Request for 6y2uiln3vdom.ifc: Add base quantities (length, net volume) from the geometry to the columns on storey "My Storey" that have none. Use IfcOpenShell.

First a look at what the model holds.

```python
import ifcopenshell
import ifcopenshell.util.element
import ifcopenshell.util.unit

model = ifcopenshell.open("6y2uiln3vdom.ifc")
print(model.schema)
for unit_type in ("LENGTHUNIT", "AREAUNIT", "VOLUMEUNIT"):
    print(unit_type, ifcopenshell.util.unit.calculate_unit_scale(model, unit_type))
storey = next(s for s in model.by_type("IfcBuildingStorey") if s.Name == "My Storey")
columns = [e for e in ifcopenshell.util.element.get_decomposition(storey) if e.is_a("IfcColumn")]
for e in sorted(columns, key=lambda e: e.id()):
    print(e.id(), e.is_a(), e.Name, list(ifcopenshell.util.element.get_psets(e, qtos_only=True)), sep=" | ")
```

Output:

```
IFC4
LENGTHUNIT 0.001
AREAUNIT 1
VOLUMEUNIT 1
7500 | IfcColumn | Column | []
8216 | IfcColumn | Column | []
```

```python
import ifcopenshell
import ifcopenshell.api.pset
import ifcopenshell.geom
import ifcopenshell.util.element
import ifcopenshell.util.shape
import ifcopenshell.util.unit

model = ifcopenshell.open("6y2uiln3vdom.ifc")
unit_scale = ifcopenshell.util.unit.calculate_unit_scale(model)
volume_scale = ifcopenshell.util.unit.calculate_unit_scale(model, "VOLUMEUNIT")
settings = ifcopenshell.geom.settings()

storey = next(s for s in model.by_type("IfcBuildingStorey") if s.Name == "My Storey")
columns = [e for e in ifcopenshell.util.element.get_decomposition(storey) if e.is_a("IfcColumn")]

for e in sorted(columns, key=lambda e: e.id()):
    if ifcopenshell.util.element.get_psets(e, qtos_only=True, should_inherit=False):
        continue
    # Geometry comes back in metres, in the element's own axes.
    shape = ifcopenshell.geom.create_shape(settings, e)
    values = {
        "Length": ifcopenshell.util.shape.get_z(shape.geometry) / unit_scale,
        "NetVolume": ifcopenshell.util.shape.get_volume(shape.geometry) / volume_scale,
    }
    qto = ifcopenshell.api.pset.add_qto(model, product=e, name="Qto_ColumnBaseQuantities")
    ifcopenshell.api.pset.edit_qto(model, qto=qto, properties=values)
    print(e.id(), {k: round(v, 3) for k, v in values.items()})

model.write("6y2uiln3vdom_v2.ifc")
```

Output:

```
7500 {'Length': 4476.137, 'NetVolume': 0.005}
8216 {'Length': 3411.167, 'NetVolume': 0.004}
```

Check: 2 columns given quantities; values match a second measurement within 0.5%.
